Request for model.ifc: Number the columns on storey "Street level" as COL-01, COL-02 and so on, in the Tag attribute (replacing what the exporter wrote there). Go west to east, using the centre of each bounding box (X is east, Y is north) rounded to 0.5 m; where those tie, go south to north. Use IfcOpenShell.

First a look at what the model holds.

```python
import ifcopenshell
import ifcopenshell.util.element
import ifcopenshell.util.placement

model = ifcopenshell.open("model.ifc")
print(model.schema)
storey = next(s for s in model.by_type("IfcBuildingStorey") if s.Name == "Street level")
columns = [e for e in ifcopenshell.util.element.get_decomposition(storey) if e.is_a("IfcColumn")]
for e in sorted(columns, key=lambda e: e.id()):
    origin = ifcopenshell.util.placement.get_local_placement(e.ObjectPlacement)[:3, 3]
    print(e.id(), e.Tag, e.Name, origin.round(2) + 0.0, sep=" | ")
```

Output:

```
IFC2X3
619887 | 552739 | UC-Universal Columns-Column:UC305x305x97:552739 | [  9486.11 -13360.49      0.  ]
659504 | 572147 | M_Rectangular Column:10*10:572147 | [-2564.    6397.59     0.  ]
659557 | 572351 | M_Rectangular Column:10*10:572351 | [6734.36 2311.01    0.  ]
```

```python
import ifcopenshell
import ifcopenshell.geom
import ifcopenshell.util.element
import ifcopenshell.util.shape

model = ifcopenshell.open("model.ifc")
settings = ifcopenshell.geom.settings()
settings.set("use-world-coords", True)


def centre(element):
    shape = ifcopenshell.geom.create_shape(settings, element)
    return ifcopenshell.util.shape.get_bbox_centroid(shape.geometry)


storey = next(s for s in model.by_type("IfcBuildingStorey") if s.Name == "Street level")
columns = [e for e in ifcopenshell.util.element.get_decomposition(storey) if e.is_a("IfcColumn")]

# Insertion points can sit at a corner or the storey origin, so sort by the geometry (in metres).
centres = {e: centre(e) for e in columns}
columns.sort(key=lambda e: (round(centres[e][0] / 0.5), centres[e][1]))

for i, e in enumerate(columns, start=1):
    number = f"COL-{i:02d}"
    e.Tag = number
    print(e.id(), number)

model.write("model_updated.ifc")
```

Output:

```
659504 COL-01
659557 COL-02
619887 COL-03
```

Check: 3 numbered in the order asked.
